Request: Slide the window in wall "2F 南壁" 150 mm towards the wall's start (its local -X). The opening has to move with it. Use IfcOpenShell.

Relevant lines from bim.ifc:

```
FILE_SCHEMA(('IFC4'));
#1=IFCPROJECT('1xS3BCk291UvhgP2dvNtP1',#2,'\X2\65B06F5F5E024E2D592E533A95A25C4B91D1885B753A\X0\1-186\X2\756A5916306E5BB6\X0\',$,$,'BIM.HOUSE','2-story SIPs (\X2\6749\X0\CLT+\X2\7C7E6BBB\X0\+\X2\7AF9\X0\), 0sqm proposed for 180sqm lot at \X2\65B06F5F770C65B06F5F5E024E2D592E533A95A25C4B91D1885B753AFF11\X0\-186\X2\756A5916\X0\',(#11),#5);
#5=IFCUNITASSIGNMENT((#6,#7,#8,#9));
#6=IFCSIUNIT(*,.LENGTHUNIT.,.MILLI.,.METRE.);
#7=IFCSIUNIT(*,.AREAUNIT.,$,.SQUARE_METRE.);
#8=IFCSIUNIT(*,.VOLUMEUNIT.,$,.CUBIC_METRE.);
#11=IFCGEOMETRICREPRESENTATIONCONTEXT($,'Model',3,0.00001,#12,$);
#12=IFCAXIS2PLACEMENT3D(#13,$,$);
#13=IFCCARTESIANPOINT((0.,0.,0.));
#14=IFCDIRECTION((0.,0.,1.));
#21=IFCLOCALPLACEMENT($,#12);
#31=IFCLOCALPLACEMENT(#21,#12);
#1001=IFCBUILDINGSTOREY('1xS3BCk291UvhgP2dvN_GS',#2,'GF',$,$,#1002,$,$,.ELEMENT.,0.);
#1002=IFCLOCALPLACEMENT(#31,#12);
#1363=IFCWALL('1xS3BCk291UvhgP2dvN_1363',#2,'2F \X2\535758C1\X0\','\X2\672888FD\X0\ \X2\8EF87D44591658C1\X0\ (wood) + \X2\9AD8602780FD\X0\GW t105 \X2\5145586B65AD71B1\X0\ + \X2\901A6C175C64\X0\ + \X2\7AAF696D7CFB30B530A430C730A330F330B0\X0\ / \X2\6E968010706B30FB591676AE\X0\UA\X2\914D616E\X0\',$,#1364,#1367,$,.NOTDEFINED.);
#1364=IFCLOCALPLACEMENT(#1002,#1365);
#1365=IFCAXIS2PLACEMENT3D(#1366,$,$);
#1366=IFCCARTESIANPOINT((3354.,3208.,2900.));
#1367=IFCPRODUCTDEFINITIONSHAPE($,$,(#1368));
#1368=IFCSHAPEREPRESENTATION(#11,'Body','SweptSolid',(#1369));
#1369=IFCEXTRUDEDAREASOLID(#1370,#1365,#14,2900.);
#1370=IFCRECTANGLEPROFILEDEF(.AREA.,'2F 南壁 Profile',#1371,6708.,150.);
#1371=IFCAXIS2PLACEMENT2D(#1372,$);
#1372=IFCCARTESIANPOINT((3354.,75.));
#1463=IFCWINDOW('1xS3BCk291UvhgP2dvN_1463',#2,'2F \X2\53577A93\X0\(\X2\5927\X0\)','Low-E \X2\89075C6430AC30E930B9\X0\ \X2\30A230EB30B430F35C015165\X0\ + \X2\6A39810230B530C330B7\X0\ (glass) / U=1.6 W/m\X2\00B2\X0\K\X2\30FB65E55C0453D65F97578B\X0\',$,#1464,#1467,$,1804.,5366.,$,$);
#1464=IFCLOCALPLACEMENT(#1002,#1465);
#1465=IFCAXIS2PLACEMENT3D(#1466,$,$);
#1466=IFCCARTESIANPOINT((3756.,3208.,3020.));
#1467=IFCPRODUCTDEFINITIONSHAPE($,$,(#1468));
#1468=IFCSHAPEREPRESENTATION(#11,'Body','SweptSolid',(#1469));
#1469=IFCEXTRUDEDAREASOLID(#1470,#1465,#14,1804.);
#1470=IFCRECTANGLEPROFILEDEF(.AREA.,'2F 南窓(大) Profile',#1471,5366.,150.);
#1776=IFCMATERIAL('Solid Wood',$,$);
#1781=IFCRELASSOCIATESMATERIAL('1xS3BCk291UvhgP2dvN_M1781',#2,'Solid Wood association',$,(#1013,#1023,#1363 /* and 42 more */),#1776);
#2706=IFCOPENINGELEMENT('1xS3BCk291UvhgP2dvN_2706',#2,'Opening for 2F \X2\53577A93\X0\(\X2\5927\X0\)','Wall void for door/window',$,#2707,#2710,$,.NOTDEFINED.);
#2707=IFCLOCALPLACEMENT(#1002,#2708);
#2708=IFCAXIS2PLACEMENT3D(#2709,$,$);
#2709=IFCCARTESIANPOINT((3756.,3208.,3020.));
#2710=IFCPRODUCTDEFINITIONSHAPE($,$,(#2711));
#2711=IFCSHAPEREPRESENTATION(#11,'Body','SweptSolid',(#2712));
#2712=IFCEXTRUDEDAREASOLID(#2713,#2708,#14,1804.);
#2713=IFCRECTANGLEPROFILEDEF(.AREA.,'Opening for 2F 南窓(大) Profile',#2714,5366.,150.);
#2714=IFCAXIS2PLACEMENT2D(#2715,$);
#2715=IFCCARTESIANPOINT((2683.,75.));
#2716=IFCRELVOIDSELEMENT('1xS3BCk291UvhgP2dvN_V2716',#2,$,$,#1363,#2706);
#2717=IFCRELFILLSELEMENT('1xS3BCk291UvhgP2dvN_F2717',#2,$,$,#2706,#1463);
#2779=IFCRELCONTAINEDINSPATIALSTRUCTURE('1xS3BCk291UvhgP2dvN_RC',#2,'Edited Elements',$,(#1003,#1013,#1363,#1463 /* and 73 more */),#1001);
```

```python
import ifcopenshell
import ifcopenshell.api.geometry
import ifcopenshell.util.placement

model = ifcopenshell.open("bim.ifc")

window = model.by_id(1463)
opening = window.FillsVoids[0].RelatingOpeningElement
wall = opening.VoidsElements[0].RelatingBuildingElement

wall_matrix = ifcopenshell.util.placement.get_local_placement(wall.ObjectPlacement)
shift = wall_matrix[:3, 0] * -150.0
before = ifcopenshell.util.placement.get_local_placement(window.ObjectPlacement)[:3, 3].copy()

# The window is not placed relative to its opening, so move both.
for product in (opening, window):
    matrix = ifcopenshell.util.placement.get_local_placement(product.ObjectPlacement)
    matrix[:3, 3] += shift
    ifcopenshell.api.geometry.edit_object_placement(model, product=product, matrix=matrix, is_si=False)

after = ifcopenshell.util.placement.get_local_placement(window.ObjectPlacement)[:3, 3]
print("window moved by", (after - before).round(3) + 0.0)

model.write("bim_edited.ifc")
```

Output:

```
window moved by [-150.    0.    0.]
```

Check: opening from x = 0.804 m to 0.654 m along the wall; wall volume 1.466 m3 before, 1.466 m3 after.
